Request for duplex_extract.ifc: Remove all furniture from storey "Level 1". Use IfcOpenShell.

First a look at what the model holds.

```python
import ifcopenshell
import ifcopenshell.util.element

model = ifcopenshell.open("duplex_extract.ifc")
print(model.schema)
storey = next(s for s in model.by_type("IfcBuildingStorey") if s.Name == "Level 1")
furniture = [e for e in ifcopenshell.util.element.get_decomposition(storey) if e.is_a("IfcFurnishingElement")]
seen = {}
for e in furniture:
    element_type = ifcopenshell.util.element.get_type(e)
    name = element_type.Name if element_type not in (None, e) else None
    seen[name] = seen.get(name, 0) + 1
for name, count in sorted(seen.items(), key=str):
    print(count, "x", name)
```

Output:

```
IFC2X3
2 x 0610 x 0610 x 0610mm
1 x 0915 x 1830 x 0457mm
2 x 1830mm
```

```python
import ifcopenshell
import ifcopenshell.api.root
import ifcopenshell.util.element

model = ifcopenshell.open("duplex_extract.ifc")

storey = next(s for s in model.by_type("IfcBuildingStorey") if s.Name == "Level 1")
furniture = [e for e in ifcopenshell.util.element.get_decomposition(storey) if e.is_a("IfcFurnishingElement")]

for e in furniture:
    ifcopenshell.api.root.remove_product(model, product=e)
print(len(furniture), "removed")

model.write("duplex_extract_rev.ifc")
```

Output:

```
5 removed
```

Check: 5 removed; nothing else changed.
